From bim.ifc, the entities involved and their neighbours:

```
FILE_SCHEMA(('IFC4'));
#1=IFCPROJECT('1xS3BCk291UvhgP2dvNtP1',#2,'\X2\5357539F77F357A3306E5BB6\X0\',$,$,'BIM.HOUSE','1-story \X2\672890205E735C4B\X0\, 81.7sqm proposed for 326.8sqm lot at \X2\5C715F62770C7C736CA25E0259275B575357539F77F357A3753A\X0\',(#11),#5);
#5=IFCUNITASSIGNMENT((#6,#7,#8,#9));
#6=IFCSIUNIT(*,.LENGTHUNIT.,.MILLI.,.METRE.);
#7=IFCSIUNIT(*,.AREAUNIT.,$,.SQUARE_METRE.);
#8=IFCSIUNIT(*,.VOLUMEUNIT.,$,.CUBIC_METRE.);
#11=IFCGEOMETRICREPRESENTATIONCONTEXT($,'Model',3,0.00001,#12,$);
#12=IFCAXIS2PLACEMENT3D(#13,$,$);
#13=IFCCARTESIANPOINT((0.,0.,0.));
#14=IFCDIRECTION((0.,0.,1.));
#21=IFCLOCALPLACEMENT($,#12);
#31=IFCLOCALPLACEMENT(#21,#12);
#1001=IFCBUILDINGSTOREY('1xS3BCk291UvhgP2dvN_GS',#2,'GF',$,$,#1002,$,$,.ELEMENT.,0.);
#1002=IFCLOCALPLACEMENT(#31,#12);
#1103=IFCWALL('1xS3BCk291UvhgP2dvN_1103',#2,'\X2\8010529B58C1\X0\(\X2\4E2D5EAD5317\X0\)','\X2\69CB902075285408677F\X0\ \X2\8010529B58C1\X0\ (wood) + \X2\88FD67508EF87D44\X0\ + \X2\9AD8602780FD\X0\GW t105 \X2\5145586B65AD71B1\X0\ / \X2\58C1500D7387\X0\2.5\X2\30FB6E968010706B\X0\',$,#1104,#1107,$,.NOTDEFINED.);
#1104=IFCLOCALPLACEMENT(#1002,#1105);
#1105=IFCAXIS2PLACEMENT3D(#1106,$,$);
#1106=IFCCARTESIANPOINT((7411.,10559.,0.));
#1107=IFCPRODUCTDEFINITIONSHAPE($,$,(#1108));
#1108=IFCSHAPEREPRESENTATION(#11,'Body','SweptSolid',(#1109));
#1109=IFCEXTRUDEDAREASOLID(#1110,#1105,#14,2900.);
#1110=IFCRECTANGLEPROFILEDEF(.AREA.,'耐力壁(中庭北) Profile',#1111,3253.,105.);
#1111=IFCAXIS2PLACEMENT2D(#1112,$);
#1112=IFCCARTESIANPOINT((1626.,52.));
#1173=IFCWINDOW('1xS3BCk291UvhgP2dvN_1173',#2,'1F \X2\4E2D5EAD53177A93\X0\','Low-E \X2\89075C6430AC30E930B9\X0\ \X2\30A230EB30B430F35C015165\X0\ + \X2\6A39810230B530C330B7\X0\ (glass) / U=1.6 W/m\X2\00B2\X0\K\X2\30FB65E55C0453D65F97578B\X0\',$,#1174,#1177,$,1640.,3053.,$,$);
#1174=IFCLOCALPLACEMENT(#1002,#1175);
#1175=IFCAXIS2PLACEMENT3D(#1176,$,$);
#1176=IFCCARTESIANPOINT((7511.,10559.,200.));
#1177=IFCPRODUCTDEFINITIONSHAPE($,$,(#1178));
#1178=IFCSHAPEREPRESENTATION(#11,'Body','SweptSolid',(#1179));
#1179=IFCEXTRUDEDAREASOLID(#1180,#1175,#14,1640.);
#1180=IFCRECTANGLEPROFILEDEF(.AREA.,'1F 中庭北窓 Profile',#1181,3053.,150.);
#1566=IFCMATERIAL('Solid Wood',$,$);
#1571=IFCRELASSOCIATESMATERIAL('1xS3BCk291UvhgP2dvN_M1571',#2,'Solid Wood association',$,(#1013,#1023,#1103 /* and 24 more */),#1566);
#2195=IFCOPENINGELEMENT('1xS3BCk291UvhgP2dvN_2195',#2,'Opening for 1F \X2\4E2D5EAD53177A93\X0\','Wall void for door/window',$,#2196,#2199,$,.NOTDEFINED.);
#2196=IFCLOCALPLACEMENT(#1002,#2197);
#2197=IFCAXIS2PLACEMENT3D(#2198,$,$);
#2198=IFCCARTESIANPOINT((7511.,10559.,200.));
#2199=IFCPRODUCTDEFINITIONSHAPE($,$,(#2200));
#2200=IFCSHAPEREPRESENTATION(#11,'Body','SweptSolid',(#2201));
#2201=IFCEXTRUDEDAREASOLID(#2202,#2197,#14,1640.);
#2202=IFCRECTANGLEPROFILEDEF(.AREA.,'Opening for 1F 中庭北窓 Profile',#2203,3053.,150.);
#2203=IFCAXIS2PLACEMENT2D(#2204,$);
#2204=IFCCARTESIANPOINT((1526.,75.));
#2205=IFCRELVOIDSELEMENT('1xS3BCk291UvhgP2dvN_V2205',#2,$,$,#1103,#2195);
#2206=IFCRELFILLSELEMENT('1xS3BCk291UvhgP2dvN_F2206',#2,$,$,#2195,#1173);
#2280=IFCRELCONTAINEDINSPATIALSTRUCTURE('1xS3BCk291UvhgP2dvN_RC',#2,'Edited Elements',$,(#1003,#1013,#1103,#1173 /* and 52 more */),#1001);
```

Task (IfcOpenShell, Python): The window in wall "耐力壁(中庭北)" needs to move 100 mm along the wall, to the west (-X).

```python
import ifcopenshell
import ifcopenshell.api.geometry
import ifcopenshell.util.placement
import ifcopenshell.util.unit

model = ifcopenshell.open("bim.ifc")
unit_scale = ifcopenshell.util.unit.calculate_unit_scale(model)

window = model.by_guid("1xS3BCk291UvhgP2dvN_1173")
opening = window.FillsVoids[0].RelatingOpeningElement
wall = opening.VoidsElements[0].RelatingBuildingElement

wall_matrix = ifcopenshell.util.placement.get_local_placement(wall.ObjectPlacement)
shift = wall_matrix[:3, 0] * -0.1 / unit_scale
before = ifcopenshell.util.placement.get_local_placement(window.ObjectPlacement)[:3, 3].copy()

# The window is not placed relative to its opening, so move both.
for product in (opening, window):
    matrix = ifcopenshell.util.placement.get_local_placement(product.ObjectPlacement)
    matrix[:3, 3] += shift
    ifcopenshell.api.geometry.edit_object_placement(model, product=product, matrix=matrix, is_si=False)

after = ifcopenshell.util.placement.get_local_placement(window.ObjectPlacement)[:3, 3]
print("window moved by", (after - before).round(3) + 0.0)

model.write("bim_v2.ifc")
```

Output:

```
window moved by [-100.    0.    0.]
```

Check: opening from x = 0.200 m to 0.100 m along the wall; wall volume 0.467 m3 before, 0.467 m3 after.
